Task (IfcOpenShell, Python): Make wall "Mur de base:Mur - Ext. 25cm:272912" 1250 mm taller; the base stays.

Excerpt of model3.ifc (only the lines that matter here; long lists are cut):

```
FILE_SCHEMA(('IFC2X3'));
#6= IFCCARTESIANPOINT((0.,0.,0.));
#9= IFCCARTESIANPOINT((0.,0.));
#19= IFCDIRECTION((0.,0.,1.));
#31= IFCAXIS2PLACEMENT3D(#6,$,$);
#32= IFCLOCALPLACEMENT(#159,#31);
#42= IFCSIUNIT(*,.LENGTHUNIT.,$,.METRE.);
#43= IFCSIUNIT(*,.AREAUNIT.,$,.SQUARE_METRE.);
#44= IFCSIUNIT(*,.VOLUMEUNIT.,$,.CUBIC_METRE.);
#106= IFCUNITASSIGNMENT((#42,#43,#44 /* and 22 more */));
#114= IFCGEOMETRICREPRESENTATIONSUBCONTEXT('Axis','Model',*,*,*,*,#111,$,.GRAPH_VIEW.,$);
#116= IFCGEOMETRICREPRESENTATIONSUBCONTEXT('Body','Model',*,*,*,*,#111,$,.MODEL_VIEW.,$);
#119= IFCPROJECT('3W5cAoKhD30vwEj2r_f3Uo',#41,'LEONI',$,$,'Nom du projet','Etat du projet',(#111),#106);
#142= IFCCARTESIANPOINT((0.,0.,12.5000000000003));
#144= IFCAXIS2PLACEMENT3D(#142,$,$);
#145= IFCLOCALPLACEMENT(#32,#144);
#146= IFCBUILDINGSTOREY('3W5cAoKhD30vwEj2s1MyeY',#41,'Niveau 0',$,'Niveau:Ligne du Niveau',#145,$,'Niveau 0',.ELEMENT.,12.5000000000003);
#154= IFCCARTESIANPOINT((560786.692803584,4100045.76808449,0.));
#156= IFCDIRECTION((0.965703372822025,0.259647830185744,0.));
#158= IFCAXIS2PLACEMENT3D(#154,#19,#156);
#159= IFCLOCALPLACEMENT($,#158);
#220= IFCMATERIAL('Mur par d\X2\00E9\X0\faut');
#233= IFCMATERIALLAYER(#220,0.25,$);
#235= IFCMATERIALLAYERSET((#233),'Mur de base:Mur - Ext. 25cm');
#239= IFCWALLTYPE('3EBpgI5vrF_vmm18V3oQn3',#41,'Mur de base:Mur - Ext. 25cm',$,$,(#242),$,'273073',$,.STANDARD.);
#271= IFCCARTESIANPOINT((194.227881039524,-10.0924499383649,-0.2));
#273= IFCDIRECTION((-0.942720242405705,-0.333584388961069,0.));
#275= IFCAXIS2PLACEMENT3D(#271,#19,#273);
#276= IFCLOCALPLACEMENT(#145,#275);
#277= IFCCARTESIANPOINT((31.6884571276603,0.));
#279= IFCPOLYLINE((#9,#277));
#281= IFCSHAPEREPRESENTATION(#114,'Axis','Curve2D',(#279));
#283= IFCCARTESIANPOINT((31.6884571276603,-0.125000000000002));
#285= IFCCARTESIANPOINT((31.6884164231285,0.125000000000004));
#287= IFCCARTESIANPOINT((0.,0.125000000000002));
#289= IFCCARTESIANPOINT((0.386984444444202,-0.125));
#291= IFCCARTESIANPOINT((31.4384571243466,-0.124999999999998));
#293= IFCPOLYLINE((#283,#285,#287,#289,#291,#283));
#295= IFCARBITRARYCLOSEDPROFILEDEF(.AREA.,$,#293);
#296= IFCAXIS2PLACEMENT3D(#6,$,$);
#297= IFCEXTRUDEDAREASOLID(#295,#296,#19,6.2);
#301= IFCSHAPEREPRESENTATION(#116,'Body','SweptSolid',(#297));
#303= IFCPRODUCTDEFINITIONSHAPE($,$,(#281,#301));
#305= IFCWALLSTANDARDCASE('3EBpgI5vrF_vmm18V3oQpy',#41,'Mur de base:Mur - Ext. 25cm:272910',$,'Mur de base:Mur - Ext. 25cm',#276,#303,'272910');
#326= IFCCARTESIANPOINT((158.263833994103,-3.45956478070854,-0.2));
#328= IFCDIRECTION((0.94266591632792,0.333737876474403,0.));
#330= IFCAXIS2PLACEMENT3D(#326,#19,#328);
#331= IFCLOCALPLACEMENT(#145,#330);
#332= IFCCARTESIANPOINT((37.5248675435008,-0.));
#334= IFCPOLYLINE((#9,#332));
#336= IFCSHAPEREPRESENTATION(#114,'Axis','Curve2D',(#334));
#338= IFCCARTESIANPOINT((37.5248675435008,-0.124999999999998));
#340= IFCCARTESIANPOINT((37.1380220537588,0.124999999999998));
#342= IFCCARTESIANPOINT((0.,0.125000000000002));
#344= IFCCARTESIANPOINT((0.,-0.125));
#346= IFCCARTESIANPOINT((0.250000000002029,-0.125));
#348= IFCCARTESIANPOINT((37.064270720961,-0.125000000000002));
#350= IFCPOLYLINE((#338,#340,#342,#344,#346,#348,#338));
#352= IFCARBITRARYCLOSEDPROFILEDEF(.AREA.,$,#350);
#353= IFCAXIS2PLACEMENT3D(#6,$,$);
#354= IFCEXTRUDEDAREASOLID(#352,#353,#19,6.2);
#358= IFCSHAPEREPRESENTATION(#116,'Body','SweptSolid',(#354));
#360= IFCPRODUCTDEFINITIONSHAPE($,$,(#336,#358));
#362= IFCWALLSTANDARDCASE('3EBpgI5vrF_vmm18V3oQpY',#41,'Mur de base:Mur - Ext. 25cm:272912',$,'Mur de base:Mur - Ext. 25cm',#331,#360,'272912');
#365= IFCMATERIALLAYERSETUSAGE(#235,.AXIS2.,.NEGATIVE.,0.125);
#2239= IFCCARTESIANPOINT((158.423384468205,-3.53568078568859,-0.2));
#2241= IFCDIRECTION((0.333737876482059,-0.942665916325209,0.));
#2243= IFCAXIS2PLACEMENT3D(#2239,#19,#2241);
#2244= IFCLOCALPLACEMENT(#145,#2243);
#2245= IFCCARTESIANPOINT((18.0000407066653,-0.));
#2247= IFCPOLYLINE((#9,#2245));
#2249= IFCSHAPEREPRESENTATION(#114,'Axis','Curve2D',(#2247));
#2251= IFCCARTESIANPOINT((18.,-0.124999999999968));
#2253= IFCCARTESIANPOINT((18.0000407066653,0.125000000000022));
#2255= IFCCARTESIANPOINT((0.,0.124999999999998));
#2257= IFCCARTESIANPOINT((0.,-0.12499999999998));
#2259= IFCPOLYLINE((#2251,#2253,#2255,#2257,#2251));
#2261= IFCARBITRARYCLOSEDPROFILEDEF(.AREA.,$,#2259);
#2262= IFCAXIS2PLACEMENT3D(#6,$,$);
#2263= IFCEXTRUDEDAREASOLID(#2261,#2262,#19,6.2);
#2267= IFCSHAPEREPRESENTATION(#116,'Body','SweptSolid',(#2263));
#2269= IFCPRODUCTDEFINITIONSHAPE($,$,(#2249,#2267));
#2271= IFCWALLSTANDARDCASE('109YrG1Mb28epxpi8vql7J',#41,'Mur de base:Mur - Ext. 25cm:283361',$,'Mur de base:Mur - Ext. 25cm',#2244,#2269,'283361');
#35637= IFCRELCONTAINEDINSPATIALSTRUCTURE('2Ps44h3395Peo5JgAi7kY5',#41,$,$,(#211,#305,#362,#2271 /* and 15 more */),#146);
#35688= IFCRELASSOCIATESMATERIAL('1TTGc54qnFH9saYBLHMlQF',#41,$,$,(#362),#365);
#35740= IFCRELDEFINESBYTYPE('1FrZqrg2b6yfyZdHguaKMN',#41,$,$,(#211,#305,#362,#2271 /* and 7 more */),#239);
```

```python
import ifcopenshell
import ifcopenshell.geom
import ifcopenshell.util.representation
import ifcopenshell.util.shape
import ifcopenshell.util.unit

model = ifcopenshell.open("model3.ifc")
unit_scale = ifcopenshell.util.unit.calculate_unit_scale(model)
settings = ifcopenshell.geom.settings()


def volume(element):
    """Net volume in cubic metres, openings subtracted."""
    shape = ifcopenshell.geom.create_shape(settings, element)
    return ifcopenshell.util.shape.get_volume(shape.geometry)


wall = model.by_guid("3EBpgI5vrF_vmm18V3oQpY")
before = volume(wall)

body = ifcopenshell.util.representation.get_representation(wall, "Model", "Body")
solid = body.Items[0]
old_height = solid.Depth
solid.Depth += 1.25 / unit_scale
after = volume(wall)

print(f"height {old_height:g} -> {solid.Depth:g}, volume {before:.3f} -> {after:.3f} m3")

model.write("model3_updated.ifc")
```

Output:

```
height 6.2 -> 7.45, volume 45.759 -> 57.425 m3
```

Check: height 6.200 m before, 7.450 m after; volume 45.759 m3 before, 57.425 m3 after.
